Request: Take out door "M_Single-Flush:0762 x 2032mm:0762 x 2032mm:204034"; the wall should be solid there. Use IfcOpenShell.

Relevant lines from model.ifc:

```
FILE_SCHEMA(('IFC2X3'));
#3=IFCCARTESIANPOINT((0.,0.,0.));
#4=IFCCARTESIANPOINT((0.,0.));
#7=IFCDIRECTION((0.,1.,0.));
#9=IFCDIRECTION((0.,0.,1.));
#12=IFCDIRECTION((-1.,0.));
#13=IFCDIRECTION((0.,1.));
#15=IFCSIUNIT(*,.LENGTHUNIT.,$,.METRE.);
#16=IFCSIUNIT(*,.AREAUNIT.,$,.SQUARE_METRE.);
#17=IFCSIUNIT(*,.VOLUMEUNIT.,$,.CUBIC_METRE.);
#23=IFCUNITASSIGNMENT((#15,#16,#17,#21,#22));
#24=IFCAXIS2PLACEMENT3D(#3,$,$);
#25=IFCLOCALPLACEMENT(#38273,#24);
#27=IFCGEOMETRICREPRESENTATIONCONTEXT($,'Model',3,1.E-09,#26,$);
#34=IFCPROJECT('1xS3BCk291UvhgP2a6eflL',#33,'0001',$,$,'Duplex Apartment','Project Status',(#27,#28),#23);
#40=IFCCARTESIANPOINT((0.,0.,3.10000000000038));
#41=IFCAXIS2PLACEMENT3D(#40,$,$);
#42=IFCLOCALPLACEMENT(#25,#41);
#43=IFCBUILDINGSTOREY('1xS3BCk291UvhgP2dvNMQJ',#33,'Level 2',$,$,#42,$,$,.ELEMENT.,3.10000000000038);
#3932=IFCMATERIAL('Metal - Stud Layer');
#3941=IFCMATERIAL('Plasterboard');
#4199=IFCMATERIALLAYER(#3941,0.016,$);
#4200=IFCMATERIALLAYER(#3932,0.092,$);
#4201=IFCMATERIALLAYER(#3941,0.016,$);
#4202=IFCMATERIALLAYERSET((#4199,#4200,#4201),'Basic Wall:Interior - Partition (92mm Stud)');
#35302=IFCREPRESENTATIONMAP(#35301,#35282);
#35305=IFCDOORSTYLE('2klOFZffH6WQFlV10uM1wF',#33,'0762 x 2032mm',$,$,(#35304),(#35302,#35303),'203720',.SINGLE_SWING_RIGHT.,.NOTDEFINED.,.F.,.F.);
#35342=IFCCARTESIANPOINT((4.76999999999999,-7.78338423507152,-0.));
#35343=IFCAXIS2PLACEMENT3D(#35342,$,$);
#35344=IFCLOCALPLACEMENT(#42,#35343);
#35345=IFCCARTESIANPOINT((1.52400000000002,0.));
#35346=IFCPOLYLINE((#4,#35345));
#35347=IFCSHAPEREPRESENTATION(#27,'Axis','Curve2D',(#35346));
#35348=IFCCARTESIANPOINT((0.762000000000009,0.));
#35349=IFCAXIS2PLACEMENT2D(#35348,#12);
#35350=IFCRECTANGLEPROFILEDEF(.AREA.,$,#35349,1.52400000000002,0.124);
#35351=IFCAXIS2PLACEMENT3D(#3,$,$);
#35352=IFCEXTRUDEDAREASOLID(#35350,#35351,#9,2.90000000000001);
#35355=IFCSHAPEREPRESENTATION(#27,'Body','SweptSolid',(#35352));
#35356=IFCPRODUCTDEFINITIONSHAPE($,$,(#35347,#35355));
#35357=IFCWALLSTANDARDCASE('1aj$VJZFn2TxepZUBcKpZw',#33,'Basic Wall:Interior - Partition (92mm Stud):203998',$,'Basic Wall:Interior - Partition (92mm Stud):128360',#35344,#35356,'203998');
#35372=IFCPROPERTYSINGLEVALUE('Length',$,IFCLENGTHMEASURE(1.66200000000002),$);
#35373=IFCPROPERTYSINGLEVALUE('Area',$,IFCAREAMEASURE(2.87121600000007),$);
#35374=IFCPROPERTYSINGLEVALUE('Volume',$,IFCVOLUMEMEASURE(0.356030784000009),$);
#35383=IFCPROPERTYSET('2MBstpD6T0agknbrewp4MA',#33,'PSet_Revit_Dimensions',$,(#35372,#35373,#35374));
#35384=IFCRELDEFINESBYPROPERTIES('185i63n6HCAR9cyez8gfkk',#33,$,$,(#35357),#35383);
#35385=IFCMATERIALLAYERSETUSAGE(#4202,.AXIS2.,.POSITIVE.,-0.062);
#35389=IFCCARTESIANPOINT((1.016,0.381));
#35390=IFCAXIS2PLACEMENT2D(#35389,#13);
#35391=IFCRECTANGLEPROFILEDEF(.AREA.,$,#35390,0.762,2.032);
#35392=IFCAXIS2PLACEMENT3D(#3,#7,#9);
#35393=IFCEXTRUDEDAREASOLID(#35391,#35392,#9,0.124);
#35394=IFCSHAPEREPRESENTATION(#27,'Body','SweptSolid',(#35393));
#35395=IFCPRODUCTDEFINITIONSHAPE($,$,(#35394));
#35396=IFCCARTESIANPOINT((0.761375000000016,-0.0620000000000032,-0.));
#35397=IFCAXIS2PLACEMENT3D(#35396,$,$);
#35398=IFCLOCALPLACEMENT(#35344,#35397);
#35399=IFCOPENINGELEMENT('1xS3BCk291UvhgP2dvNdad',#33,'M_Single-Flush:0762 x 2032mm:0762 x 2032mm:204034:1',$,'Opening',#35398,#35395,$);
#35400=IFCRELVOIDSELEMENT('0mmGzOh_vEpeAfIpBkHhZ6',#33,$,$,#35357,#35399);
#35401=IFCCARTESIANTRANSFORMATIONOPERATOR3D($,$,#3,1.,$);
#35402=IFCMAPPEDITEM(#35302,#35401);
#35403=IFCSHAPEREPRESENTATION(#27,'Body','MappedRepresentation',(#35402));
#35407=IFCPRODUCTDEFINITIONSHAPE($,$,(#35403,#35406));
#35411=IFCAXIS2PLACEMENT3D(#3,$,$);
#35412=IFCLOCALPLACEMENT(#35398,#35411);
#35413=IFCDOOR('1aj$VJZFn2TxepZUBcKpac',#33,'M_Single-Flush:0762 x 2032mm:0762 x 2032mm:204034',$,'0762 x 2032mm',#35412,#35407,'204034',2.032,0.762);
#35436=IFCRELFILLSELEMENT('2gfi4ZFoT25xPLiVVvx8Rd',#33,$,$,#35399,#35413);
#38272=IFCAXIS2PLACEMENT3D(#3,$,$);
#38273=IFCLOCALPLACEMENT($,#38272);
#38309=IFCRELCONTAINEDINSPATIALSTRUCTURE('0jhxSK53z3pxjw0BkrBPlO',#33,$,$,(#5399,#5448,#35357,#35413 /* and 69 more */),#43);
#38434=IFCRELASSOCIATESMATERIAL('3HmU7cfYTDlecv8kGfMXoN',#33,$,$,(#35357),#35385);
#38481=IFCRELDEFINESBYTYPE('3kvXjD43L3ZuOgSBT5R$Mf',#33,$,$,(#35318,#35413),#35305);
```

```python
import ifcopenshell
import ifcopenshell.api.feature
import ifcopenshell.api.pset
import ifcopenshell.api.root
import ifcopenshell.geom
import ifcopenshell.util.element
import ifcopenshell.util.shape
import ifcopenshell.util.unit

model = ifcopenshell.open("model.ifc")
area_scale = ifcopenshell.util.unit.calculate_unit_scale(model, "AREAUNIT")
volume_scale = ifcopenshell.util.unit.calculate_unit_scale(model, "VOLUMEUNIT")
settings = ifcopenshell.geom.settings()


def volume(element):
    """Net volume in cubic metres, openings subtracted."""
    shape = ifcopenshell.geom.create_shape(settings, element)
    return ifcopenshell.util.shape.get_volume(shape.geometry)


door = model.by_guid("1aj$VJZFn2TxepZUBcKpac")
opening = door.FillsVoids[0].RelatingOpeningElement
wall = opening.VoidsElements[0].RelatingBuildingElement
before = volume(wall)

ifcopenshell.api.root.remove_product(model, product=door)
ifcopenshell.api.feature.remove_feature(model, feature=opening)

after = volume(wall)
thickness = 0.124  # wall thickness in metres

# Update the wall's stored quantities.
pset = model.by_id(ifcopenshell.util.element.get_pset(wall, "PSet_Revit_Dimensions", should_inherit=False)["id"])
ifcopenshell.api.pset.edit_pset(model, pset=pset, properties={
    "Area": model.create_entity("IfcAreaMeasure", after / thickness / area_scale),
    "Volume": model.create_entity("IfcVolumeMeasure", after / volume_scale),
})

print(f"wall volume {before:.3f} -> {after:.3f} m3")

model.write("model-out.ifc")
```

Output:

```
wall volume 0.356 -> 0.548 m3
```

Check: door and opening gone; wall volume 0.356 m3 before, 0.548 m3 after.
